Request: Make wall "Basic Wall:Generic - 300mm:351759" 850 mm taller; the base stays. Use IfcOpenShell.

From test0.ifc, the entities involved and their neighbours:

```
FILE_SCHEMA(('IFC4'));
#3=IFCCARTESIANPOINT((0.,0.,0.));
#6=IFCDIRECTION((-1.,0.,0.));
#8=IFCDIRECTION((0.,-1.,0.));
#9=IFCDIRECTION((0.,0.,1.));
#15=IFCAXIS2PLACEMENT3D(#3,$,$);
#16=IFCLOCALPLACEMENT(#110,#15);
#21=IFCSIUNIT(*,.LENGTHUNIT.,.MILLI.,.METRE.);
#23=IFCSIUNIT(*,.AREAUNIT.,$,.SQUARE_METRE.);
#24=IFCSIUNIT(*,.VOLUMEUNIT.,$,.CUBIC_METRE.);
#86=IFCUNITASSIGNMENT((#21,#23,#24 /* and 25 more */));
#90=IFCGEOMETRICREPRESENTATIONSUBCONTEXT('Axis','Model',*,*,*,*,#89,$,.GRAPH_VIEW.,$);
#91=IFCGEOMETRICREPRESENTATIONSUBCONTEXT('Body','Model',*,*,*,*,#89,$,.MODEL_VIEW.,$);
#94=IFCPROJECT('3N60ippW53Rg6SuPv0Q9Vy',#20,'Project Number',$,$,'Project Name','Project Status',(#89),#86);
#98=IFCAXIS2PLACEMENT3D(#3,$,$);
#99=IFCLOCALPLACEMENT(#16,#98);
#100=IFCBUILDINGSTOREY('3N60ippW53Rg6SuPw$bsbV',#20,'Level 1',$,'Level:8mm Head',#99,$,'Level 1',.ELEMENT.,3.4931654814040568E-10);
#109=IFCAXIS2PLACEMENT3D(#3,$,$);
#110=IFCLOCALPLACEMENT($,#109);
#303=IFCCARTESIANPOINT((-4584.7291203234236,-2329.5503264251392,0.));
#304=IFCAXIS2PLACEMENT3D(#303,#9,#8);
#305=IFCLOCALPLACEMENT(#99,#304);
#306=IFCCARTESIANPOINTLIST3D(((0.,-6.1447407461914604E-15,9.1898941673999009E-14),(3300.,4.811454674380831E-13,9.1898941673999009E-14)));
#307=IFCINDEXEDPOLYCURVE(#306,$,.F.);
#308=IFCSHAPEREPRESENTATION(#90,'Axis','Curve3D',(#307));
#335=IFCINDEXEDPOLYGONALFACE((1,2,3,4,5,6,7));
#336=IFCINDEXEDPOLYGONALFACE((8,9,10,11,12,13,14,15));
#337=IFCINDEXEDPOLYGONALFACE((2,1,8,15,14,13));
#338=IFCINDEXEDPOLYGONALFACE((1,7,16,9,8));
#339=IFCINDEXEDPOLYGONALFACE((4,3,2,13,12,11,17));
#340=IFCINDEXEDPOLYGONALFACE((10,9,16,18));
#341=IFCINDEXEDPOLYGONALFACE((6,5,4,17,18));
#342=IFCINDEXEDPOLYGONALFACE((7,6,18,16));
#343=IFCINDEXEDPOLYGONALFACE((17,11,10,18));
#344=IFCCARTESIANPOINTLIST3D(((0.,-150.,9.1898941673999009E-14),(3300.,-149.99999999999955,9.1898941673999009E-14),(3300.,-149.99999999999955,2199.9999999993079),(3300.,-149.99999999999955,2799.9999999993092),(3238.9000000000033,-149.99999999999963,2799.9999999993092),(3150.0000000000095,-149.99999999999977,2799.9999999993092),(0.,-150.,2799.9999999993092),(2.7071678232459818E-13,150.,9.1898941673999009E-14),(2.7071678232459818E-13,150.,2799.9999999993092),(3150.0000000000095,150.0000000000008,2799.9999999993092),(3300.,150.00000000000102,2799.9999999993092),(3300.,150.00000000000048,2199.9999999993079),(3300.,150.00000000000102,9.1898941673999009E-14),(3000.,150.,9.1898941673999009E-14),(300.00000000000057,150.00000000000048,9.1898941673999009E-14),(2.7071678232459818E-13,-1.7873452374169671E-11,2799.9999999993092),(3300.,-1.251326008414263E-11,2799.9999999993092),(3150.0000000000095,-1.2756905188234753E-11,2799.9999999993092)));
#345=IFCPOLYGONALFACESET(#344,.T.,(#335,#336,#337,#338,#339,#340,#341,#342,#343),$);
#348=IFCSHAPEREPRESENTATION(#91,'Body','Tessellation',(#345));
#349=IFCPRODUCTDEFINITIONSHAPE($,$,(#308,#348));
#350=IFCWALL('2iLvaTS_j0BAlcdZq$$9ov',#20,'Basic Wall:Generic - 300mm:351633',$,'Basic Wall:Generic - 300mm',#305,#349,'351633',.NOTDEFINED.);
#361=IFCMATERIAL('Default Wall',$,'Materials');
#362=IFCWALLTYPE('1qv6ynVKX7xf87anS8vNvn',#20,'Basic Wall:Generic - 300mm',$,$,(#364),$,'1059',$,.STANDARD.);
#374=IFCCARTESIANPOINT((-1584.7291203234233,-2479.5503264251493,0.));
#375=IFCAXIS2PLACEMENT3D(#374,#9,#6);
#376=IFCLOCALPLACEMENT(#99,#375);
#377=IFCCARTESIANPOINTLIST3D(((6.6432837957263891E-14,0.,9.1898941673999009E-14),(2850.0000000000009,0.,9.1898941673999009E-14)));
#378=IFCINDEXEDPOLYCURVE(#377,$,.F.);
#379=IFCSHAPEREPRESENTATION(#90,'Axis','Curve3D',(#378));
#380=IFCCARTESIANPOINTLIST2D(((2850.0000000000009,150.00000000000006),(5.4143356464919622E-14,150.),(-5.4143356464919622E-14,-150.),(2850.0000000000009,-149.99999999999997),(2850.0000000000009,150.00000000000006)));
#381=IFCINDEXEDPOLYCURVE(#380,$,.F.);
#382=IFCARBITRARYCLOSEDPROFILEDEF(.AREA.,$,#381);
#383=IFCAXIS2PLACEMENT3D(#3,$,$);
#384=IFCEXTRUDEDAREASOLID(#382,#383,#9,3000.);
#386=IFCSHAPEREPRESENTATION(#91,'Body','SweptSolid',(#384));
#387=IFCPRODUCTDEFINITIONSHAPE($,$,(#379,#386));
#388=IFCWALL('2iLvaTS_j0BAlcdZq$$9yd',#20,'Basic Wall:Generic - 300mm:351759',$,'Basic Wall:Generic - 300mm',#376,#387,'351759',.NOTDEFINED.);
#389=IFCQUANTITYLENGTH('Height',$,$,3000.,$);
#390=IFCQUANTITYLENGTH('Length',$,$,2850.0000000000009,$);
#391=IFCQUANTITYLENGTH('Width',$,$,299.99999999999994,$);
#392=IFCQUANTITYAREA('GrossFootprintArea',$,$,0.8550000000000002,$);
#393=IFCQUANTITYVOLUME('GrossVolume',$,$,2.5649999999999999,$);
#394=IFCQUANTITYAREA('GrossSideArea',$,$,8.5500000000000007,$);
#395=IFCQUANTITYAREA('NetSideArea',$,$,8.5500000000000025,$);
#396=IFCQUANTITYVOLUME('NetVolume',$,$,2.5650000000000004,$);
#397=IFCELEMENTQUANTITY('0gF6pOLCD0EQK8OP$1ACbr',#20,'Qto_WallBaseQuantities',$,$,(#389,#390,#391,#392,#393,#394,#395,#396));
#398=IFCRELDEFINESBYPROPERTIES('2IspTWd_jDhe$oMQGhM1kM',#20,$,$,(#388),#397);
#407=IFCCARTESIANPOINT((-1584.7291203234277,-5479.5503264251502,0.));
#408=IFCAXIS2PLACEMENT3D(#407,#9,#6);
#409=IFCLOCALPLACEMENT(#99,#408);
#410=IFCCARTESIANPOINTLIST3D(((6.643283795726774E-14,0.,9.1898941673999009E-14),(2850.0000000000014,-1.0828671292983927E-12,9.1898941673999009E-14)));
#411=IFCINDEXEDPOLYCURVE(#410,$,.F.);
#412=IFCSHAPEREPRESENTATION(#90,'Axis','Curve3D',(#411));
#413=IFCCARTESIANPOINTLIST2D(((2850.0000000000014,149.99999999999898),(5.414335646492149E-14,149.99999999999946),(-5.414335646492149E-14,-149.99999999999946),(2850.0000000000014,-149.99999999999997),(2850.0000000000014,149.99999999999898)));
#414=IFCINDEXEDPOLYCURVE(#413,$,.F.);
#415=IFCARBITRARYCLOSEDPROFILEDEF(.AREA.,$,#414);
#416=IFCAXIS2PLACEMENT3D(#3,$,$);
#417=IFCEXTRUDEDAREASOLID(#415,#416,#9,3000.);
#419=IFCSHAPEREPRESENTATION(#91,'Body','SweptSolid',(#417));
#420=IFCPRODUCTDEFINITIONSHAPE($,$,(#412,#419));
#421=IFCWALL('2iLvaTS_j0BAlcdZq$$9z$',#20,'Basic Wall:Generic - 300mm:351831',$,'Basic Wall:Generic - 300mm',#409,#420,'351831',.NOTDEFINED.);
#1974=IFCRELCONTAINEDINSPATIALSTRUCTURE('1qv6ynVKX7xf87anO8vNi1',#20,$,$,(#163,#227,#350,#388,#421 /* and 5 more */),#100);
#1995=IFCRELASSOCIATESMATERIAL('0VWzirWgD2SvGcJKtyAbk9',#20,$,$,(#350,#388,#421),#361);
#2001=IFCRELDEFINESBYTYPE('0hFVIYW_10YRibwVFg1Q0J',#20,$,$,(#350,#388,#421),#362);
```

```python
import ifcopenshell
import ifcopenshell.api.pset
import ifcopenshell.geom
import ifcopenshell.util.element
import ifcopenshell.util.representation
import ifcopenshell.util.shape
import ifcopenshell.util.unit

model = ifcopenshell.open("test0.ifc")
unit_scale = ifcopenshell.util.unit.calculate_unit_scale(model)
area_scale = ifcopenshell.util.unit.calculate_unit_scale(model, "AREAUNIT")
volume_scale = ifcopenshell.util.unit.calculate_unit_scale(model, "VOLUMEUNIT")
settings = ifcopenshell.geom.settings()


def volume(element):
    """Net volume in cubic metres, openings subtracted."""
    shape = ifcopenshell.geom.create_shape(settings, element)
    return ifcopenshell.util.shape.get_volume(shape.geometry)


wall = model.by_guid("2iLvaTS_j0BAlcdZq$$9yd")
before = volume(wall)

body = ifcopenshell.util.representation.get_representation(wall, "Model", "Body")
solid = body.Items[0]
old_height = solid.Depth
solid.Depth += 0.85 / unit_scale
after = volume(wall)
thickness = 0.3  # wall thickness in metres

# Update the stored height, areas and volumes.
qto = model.by_id(ifcopenshell.util.element.get_pset(wall, "Qto_WallBaseQuantities", should_inherit=False)["id"])
ifcopenshell.api.pset.edit_qto(model, qto=qto, properties={
    "Height": solid.Depth,
    "GrossVolume": ifcopenshell.util.element.get_pset(wall, "Qto_WallBaseQuantities", "GrossVolume") * solid.Depth / old_height,
    "GrossSideArea": ifcopenshell.util.element.get_pset(wall, "Qto_WallBaseQuantities", "GrossSideArea") * solid.Depth / old_height,
    "NetSideArea": after / thickness / area_scale,
    "NetVolume": after / volume_scale,
})

print(f"height {old_height:g} -> {solid.Depth:g}, volume {before:.3f} -> {after:.3f} m3")

model.write("test0_v2.ifc")
```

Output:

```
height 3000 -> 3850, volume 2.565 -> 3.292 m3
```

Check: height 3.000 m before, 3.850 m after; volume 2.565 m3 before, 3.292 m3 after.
